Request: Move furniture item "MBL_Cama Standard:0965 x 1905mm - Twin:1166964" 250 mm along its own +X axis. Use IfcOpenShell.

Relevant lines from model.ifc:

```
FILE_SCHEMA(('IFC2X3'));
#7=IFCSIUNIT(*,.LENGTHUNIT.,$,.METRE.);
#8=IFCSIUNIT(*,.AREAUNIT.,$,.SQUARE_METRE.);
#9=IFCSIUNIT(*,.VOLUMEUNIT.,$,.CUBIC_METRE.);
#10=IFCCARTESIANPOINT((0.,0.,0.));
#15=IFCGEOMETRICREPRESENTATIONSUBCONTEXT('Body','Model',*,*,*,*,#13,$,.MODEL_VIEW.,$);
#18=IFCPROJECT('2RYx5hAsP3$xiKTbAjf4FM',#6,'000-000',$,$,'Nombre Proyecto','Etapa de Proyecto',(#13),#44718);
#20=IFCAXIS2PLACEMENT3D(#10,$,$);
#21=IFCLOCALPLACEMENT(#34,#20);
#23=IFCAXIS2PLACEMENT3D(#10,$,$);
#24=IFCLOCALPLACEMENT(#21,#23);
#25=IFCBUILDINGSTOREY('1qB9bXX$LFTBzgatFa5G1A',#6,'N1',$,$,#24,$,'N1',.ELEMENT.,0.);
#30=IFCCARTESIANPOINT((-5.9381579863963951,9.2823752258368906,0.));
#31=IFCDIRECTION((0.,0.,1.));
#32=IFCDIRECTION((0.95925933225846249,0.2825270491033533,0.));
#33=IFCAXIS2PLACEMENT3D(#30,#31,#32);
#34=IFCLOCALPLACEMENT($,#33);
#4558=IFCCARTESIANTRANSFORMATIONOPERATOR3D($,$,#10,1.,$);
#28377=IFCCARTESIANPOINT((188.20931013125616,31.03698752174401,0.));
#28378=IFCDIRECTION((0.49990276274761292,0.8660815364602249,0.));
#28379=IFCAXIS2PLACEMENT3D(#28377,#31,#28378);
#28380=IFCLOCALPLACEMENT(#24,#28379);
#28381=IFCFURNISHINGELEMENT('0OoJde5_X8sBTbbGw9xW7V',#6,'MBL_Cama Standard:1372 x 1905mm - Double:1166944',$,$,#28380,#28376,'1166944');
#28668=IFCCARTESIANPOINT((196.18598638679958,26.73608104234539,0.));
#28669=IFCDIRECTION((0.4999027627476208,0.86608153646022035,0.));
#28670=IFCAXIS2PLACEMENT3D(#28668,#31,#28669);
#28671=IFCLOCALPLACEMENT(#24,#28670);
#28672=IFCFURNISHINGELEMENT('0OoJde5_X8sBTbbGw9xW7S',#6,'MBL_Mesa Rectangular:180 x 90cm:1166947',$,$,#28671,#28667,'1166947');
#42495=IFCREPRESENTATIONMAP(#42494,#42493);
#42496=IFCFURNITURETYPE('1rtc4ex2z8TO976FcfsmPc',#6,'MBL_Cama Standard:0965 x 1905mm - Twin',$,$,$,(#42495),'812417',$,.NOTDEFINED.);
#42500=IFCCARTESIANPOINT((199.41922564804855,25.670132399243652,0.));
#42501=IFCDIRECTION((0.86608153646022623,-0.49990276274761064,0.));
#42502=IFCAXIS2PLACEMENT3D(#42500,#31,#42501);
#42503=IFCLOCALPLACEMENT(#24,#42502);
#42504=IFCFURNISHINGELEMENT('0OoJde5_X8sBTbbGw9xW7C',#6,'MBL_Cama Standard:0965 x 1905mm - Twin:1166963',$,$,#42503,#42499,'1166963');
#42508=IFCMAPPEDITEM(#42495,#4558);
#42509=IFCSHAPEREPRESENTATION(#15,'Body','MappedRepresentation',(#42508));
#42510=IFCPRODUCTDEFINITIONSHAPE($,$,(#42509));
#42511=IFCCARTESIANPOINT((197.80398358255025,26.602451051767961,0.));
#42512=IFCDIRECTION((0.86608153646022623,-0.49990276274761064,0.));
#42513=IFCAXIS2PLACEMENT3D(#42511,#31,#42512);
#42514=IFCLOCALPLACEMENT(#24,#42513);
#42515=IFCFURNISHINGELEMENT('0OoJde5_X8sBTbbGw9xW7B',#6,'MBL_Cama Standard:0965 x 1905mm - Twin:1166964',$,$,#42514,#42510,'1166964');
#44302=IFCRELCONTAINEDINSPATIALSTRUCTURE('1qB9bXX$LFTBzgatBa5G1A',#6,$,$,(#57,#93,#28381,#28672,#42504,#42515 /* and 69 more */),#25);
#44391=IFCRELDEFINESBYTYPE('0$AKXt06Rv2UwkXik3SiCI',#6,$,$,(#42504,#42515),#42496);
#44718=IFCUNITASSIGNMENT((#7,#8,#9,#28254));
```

```python
import ifcopenshell
import ifcopenshell.api.geometry
import ifcopenshell.util.placement
import ifcopenshell.util.unit

model = ifcopenshell.open("model.ifc")
unit_scale = ifcopenshell.util.unit.calculate_unit_scale(model)

item = model.by_guid("0OoJde5_X8sBTbbGw9xW7B")
matrix = ifcopenshell.util.placement.get_local_placement(item.ObjectPlacement)
matrix[:3, 3] += matrix[:3, 0] * 0.25 / unit_scale
ifcopenshell.api.geometry.edit_object_placement(model, product=item, matrix=matrix, is_si=False)

print(ifcopenshell.util.placement.get_local_placement(item.ObjectPlacement).round(3) + 0.0)

model.write("model_edited.ifc")
```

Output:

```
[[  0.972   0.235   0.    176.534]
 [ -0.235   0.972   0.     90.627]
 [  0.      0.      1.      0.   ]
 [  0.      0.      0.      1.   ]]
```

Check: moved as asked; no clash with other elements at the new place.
